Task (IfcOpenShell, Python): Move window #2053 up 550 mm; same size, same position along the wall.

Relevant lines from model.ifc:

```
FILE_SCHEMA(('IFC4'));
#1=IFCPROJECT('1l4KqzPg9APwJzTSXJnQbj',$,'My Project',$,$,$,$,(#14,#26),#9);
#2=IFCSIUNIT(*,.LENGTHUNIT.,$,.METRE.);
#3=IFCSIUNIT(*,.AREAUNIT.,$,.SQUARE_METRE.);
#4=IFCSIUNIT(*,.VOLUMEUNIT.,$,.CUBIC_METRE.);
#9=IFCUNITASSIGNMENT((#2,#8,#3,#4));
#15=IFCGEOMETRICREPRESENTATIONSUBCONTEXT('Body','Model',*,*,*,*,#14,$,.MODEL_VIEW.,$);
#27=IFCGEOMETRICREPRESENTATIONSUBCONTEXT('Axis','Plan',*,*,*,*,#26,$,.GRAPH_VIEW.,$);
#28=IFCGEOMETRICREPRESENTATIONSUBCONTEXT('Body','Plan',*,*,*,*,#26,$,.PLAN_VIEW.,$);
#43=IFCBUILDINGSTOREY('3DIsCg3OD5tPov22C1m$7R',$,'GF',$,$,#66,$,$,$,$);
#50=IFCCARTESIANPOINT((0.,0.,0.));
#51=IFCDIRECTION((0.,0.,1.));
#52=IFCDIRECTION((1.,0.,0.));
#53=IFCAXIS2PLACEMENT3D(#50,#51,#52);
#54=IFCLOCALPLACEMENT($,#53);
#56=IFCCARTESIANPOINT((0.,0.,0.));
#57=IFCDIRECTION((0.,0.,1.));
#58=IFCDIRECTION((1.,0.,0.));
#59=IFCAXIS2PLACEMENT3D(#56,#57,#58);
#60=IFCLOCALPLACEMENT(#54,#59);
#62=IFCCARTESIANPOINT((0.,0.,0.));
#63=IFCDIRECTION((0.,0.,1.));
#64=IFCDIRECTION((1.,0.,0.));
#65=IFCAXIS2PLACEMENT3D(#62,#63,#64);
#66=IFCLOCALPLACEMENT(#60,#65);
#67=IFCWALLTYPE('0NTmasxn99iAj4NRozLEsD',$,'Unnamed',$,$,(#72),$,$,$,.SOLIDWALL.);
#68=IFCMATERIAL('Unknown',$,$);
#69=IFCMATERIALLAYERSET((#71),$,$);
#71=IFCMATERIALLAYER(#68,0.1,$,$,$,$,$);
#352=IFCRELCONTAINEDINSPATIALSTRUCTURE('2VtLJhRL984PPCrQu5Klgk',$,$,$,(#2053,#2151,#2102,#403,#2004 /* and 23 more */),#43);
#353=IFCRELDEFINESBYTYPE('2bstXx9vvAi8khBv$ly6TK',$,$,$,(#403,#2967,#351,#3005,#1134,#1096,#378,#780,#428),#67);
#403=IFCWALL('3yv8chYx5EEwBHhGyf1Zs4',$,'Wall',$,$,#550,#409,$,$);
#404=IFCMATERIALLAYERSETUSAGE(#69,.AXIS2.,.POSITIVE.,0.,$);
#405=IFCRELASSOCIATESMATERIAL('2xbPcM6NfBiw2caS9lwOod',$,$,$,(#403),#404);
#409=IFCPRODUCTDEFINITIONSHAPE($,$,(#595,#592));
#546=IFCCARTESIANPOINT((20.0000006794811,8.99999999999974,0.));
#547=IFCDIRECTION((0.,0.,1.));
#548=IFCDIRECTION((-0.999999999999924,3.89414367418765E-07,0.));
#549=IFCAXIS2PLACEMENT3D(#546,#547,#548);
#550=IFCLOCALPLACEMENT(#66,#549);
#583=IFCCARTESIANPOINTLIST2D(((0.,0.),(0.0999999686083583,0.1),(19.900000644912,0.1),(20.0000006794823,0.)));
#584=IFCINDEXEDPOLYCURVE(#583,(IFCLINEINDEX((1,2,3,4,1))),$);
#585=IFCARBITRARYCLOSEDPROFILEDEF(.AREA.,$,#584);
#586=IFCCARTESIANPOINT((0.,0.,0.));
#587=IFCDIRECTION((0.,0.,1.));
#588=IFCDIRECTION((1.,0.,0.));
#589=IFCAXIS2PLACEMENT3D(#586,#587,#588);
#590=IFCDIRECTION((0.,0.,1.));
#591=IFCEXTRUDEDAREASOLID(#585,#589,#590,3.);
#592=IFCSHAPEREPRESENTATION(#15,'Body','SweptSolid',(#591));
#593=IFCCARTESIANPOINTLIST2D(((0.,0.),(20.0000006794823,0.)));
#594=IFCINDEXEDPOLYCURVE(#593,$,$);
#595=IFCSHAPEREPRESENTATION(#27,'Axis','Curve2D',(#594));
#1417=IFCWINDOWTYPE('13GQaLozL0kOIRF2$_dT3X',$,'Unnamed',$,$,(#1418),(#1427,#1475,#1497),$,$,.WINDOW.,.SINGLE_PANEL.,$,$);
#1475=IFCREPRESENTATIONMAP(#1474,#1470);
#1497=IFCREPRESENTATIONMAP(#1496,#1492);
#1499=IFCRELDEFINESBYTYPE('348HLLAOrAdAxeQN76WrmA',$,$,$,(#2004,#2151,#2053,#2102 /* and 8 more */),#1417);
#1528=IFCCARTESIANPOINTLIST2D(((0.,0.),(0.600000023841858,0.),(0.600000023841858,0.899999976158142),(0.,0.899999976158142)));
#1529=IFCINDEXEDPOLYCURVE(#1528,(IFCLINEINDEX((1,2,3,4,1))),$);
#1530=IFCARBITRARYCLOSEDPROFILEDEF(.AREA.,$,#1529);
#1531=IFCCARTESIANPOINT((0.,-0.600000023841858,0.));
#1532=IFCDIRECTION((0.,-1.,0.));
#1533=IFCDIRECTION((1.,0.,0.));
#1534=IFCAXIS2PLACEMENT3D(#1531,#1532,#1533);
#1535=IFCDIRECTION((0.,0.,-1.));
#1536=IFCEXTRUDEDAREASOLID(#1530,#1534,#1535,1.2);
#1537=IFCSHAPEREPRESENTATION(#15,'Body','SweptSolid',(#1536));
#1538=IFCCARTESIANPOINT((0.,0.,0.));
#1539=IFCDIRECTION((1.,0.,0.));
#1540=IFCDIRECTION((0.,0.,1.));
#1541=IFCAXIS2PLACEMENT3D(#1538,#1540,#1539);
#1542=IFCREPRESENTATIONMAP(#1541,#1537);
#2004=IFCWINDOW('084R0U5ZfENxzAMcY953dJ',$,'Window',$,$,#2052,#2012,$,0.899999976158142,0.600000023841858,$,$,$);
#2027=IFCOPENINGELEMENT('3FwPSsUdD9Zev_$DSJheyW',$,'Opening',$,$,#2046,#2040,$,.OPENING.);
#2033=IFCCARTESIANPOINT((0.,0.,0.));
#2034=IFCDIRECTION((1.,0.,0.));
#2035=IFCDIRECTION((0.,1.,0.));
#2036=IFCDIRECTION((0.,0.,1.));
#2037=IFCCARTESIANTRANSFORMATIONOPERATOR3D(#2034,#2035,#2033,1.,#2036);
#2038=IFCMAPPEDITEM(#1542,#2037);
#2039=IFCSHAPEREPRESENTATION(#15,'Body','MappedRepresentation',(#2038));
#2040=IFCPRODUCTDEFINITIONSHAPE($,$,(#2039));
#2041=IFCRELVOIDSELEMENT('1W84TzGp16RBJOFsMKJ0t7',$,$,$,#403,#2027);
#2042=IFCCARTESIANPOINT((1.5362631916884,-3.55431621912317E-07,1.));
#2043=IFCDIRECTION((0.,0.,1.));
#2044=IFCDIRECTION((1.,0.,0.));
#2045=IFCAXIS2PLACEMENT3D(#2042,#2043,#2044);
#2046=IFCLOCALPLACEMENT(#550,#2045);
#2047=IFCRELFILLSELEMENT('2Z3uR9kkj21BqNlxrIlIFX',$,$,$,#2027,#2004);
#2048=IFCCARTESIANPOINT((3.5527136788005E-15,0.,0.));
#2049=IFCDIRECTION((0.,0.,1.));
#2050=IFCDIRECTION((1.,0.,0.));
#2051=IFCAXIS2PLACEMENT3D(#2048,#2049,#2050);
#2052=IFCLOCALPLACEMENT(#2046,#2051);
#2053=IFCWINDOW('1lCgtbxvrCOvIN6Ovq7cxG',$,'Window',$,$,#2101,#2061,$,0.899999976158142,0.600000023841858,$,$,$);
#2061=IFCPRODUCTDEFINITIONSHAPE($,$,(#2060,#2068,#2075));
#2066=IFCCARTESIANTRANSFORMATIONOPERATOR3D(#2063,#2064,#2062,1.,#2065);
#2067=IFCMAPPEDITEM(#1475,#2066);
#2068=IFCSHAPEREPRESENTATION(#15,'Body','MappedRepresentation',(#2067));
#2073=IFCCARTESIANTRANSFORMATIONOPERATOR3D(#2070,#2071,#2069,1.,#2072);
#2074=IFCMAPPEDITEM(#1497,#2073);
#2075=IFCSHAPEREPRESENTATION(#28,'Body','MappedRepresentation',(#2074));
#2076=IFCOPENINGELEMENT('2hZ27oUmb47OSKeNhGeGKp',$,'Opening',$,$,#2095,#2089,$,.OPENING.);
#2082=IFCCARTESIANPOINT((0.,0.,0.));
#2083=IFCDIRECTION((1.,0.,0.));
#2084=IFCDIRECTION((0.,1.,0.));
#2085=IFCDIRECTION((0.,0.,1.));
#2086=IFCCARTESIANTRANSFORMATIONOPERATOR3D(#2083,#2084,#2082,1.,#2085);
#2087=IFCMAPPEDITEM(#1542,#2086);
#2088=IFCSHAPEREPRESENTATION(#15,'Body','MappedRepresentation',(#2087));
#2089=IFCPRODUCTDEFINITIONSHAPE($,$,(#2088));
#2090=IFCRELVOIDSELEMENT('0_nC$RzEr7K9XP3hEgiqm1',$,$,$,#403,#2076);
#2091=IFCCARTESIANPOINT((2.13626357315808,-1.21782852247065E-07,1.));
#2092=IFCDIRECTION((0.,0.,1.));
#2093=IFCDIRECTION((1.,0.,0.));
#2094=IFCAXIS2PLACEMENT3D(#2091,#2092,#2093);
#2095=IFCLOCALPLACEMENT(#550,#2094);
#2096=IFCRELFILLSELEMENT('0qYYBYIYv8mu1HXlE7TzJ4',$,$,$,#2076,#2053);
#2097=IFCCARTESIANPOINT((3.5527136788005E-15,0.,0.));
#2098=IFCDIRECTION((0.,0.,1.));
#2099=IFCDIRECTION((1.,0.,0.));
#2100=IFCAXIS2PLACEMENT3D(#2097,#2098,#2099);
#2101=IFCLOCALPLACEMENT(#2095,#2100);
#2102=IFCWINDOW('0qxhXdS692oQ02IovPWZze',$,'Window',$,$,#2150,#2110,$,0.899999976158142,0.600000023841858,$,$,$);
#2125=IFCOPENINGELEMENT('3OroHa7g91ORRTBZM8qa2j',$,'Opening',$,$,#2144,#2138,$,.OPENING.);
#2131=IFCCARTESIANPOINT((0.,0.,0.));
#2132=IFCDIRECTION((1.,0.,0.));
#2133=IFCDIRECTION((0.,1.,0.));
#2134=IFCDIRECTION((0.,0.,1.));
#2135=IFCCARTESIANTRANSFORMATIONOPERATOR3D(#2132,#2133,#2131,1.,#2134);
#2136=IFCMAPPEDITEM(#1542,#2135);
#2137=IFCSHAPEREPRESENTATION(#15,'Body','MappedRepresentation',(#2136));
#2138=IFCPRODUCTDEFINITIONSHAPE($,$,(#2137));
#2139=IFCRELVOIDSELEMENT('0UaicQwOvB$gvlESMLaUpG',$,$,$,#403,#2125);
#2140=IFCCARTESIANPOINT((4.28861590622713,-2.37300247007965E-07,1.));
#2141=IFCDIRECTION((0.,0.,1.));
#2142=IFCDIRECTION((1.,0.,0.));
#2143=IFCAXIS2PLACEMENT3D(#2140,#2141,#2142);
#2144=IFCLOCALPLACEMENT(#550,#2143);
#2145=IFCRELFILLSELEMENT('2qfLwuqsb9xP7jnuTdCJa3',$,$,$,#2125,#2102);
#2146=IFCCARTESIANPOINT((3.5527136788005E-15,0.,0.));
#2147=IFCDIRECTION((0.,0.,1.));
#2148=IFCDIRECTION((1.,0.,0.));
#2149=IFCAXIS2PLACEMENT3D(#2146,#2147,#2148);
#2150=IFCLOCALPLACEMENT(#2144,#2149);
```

```python
import numpy as np
import ifcopenshell
import ifcopenshell.api.geometry
import ifcopenshell.util.placement
import ifcopenshell.util.unit

model = ifcopenshell.open("model.ifc")
unit_scale = ifcopenshell.util.unit.calculate_unit_scale(model)

window = model.by_id(2053)
opening = window.FillsVoids[0].RelatingOpeningElement
dz = 0.55

shift = np.array([0.0, 0.0, dz])
# The window is placed relative to its opening, so it follows when the opening moves.
matrix = ifcopenshell.util.placement.get_local_placement(opening.ObjectPlacement)
matrix[:3, 3] += shift
ifcopenshell.api.geometry.edit_object_placement(
    model, product=opening, matrix=matrix, is_si=False, should_transform_children=True
)

print(f"moved by {dz * unit_scale:+.3f} m")

model.write("model-out.ifc")
```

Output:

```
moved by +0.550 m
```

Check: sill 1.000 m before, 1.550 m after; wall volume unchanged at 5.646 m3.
